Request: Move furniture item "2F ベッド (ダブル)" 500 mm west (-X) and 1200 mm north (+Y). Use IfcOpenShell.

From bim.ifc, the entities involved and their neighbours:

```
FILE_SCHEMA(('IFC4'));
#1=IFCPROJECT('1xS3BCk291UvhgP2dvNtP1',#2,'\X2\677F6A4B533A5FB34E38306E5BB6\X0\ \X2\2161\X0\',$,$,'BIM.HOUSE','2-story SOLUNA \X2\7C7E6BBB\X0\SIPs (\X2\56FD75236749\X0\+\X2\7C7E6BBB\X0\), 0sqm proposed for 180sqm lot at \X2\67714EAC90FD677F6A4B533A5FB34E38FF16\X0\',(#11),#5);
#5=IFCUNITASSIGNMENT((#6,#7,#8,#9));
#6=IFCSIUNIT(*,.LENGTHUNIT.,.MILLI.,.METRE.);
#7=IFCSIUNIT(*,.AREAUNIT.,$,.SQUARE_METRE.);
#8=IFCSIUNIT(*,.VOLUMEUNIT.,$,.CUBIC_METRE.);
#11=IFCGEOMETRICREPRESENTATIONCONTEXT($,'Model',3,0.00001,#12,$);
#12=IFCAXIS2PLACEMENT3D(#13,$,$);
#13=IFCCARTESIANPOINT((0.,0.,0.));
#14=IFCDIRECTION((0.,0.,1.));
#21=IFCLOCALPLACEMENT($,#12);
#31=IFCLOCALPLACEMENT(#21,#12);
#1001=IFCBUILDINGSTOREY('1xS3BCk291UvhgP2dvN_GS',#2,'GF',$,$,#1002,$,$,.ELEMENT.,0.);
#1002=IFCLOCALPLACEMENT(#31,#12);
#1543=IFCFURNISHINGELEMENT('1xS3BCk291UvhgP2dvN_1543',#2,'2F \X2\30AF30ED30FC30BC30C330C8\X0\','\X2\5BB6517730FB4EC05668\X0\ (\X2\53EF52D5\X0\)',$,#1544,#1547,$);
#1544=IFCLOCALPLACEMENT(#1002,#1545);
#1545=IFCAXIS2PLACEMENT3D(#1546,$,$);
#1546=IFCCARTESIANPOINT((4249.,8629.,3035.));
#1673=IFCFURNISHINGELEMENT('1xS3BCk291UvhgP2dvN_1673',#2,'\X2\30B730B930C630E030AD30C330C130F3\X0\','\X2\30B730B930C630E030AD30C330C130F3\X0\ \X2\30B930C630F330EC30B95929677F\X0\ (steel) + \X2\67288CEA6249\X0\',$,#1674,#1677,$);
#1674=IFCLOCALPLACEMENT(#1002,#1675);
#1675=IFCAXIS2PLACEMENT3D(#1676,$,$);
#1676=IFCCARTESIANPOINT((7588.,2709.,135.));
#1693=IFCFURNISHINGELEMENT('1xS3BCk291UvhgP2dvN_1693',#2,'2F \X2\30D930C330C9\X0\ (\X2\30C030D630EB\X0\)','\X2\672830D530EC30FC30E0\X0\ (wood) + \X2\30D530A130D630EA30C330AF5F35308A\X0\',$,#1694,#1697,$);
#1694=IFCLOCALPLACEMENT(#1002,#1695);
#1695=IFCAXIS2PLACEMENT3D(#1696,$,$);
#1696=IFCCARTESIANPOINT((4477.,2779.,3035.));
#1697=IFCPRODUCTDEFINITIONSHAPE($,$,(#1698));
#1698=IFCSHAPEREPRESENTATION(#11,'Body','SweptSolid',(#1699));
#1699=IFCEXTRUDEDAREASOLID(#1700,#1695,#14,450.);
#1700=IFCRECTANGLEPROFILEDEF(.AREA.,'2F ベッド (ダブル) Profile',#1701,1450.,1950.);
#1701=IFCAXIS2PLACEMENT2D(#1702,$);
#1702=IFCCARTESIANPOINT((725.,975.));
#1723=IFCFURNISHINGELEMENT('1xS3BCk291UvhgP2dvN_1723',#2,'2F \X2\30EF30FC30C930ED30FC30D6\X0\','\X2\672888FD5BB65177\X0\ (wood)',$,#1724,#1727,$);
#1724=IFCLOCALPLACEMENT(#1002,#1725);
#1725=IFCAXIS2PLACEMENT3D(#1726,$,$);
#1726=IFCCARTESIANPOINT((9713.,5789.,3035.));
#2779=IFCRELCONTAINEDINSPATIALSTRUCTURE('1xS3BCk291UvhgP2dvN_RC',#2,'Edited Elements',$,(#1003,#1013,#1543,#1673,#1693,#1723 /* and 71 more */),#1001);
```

```python
import ifcopenshell
import ifcopenshell.api.geometry
import ifcopenshell.util.placement
import ifcopenshell.util.unit

model = ifcopenshell.open("bim.ifc")
unit_scale = ifcopenshell.util.unit.calculate_unit_scale(model)

item = model.by_guid("1xS3BCk291UvhgP2dvN_1693")
matrix = ifcopenshell.util.placement.get_local_placement(item.ObjectPlacement)
matrix[0, 3] -= 0.5 / unit_scale
matrix[1, 3] += 1.2 / unit_scale
ifcopenshell.api.geometry.edit_object_placement(model, product=item, matrix=matrix, is_si=False)

print(ifcopenshell.util.placement.get_local_placement(item.ObjectPlacement).round(3) + 0.0)

model.write("bim_rev.ifc")
```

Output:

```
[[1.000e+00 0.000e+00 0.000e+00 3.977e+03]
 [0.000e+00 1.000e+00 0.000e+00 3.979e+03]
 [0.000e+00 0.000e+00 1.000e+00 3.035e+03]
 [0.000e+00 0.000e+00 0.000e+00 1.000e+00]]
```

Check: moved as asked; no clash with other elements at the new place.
